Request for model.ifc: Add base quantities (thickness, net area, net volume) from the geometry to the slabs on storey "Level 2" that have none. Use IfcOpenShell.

First a look at what the model holds.

```python
import ifcopenshell
import ifcopenshell.util.element
import ifcopenshell.util.unit

model = ifcopenshell.open("model.ifc")
print(model.schema)
for unit_type in ("LENGTHUNIT", "AREAUNIT", "VOLUMEUNIT"):
    print(unit_type, ifcopenshell.util.unit.calculate_unit_scale(model, unit_type))
storey = next(s for s in model.by_type("IfcBuildingStorey") if s.Name == "Level 2")
slabs = [e for e in ifcopenshell.util.element.get_decomposition(storey) if e.is_a("IfcSlab")]
for e in sorted(slabs, key=lambda e: e.id()):
    print(e.id(), e.is_a(), e.Name, list(ifcopenshell.util.element.get_psets(e, qtos_only=True)), sep=" | ")
```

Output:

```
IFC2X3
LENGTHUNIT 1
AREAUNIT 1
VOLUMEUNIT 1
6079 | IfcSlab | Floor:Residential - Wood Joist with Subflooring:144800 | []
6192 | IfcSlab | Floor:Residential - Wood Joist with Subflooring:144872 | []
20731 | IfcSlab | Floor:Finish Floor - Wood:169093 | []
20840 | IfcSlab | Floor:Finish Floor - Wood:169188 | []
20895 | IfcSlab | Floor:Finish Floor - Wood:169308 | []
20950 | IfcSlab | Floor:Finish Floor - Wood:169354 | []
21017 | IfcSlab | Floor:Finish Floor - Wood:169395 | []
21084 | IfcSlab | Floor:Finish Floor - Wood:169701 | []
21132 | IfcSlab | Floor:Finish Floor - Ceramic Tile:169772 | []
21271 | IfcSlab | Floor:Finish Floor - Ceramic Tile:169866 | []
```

```python
import ifcopenshell
import ifcopenshell.api.pset
import ifcopenshell.geom
import ifcopenshell.util.element
import ifcopenshell.util.shape
import ifcopenshell.util.unit

model = ifcopenshell.open("model.ifc")
unit_scale = ifcopenshell.util.unit.calculate_unit_scale(model)
area_scale = ifcopenshell.util.unit.calculate_unit_scale(model, "AREAUNIT")
volume_scale = ifcopenshell.util.unit.calculate_unit_scale(model, "VOLUMEUNIT")
settings = ifcopenshell.geom.settings()

storey = next(s for s in model.by_type("IfcBuildingStorey") if s.Name == "Level 2")
slabs = [e for e in ifcopenshell.util.element.get_decomposition(storey) if e.is_a("IfcSlab")]

for e in sorted(slabs, key=lambda e: e.id()):
    if ifcopenshell.util.element.get_psets(e, qtos_only=True, should_inherit=False):
        continue
    # Geometry comes back in metres, in the element's own axes.
    shape = ifcopenshell.geom.create_shape(settings, e)
    values = {
        "Width": ifcopenshell.util.shape.get_z(shape.geometry) / unit_scale,
        "NetArea": ifcopenshell.util.shape.get_footprint_area(shape.geometry) / area_scale,
        "NetVolume": ifcopenshell.util.shape.get_volume(shape.geometry) / volume_scale,
    }
    qto = ifcopenshell.api.pset.add_qto(model, product=e, name="BaseQuantities")
    ifcopenshell.api.pset.edit_qto(model, qto=qto, properties=values)
    print(e.id(), {k: round(v, 3) for k, v in values.items()})

model.write("model_updated.ifc")
```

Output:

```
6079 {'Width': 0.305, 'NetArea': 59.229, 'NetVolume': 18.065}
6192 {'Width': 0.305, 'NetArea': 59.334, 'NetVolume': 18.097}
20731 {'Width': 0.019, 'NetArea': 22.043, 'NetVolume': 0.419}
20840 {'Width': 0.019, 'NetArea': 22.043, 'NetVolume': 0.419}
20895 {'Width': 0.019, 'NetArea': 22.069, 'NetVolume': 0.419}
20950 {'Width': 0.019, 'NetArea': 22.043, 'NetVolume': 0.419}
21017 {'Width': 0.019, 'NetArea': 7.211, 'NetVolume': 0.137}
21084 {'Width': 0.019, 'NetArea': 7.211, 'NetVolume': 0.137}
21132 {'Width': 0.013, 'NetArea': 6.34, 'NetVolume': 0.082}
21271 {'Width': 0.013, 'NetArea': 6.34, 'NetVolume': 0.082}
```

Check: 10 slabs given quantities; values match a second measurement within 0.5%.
